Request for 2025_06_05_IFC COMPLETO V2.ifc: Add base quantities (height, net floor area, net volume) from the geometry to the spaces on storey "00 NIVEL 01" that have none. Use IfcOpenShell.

First a look at what the model holds.

```python
import ifcopenshell
import ifcopenshell.util.element
import ifcopenshell.util.unit

model = ifcopenshell.open("2025_06_05_IFC COMPLETO V2.ifc")
print(model.schema)
for unit_type in ("LENGTHUNIT", "AREAUNIT", "VOLUMEUNIT"):
    print(unit_type, ifcopenshell.util.unit.calculate_unit_scale(model, unit_type))
storey = next(s for s in model.by_type("IfcBuildingStorey") if s.Name == "00 NIVEL 01")
spaces = [e for e in ifcopenshell.util.element.get_decomposition(storey) if e.is_a("IfcSpace")]
for e in sorted(spaces, key=lambda e: e.id()):
    print(e.id(), e.is_a(), e.Name, list(ifcopenshell.util.element.get_psets(e, qtos_only=True)), sep=" | ")
```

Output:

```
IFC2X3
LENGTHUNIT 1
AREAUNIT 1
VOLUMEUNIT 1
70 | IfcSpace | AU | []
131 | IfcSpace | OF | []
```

```python
import ifcopenshell
import ifcopenshell.api.pset
import ifcopenshell.geom
import ifcopenshell.util.element
import ifcopenshell.util.shape
import ifcopenshell.util.unit

model = ifcopenshell.open("2025_06_05_IFC COMPLETO V2.ifc")
unit_scale = ifcopenshell.util.unit.calculate_unit_scale(model)
area_scale = ifcopenshell.util.unit.calculate_unit_scale(model, "AREAUNIT")
volume_scale = ifcopenshell.util.unit.calculate_unit_scale(model, "VOLUMEUNIT")
settings = ifcopenshell.geom.settings()

storey = next(s for s in model.by_type("IfcBuildingStorey") if s.Name == "00 NIVEL 01")
spaces = [e for e in ifcopenshell.util.element.get_decomposition(storey) if e.is_a("IfcSpace")]

for e in sorted(spaces, key=lambda e: e.id()):
    if ifcopenshell.util.element.get_psets(e, qtos_only=True, should_inherit=False):
        continue
    # Geometry comes back in metres, in the element's own axes.
    shape = ifcopenshell.geom.create_shape(settings, e)
    values = {
        "Height": ifcopenshell.util.shape.get_z(shape.geometry) / unit_scale,
        "NetFloorArea": ifcopenshell.util.shape.get_footprint_area(shape.geometry) / area_scale,
        "NetVolume": ifcopenshell.util.shape.get_volume(shape.geometry) / volume_scale,
    }
    qto = ifcopenshell.api.pset.add_qto(model, product=e, name="BaseQuantities")
    ifcopenshell.api.pset.edit_qto(model, qto=qto, properties=values)
    print(e.id(), {k: round(v, 3) for k, v in values.items()})

model.write("2025_06_05_IFC COMPLETO V2_v2.ifc")
```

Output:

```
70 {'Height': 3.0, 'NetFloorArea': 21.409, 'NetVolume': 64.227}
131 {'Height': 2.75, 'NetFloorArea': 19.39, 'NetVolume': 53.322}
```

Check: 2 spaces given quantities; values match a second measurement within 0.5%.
